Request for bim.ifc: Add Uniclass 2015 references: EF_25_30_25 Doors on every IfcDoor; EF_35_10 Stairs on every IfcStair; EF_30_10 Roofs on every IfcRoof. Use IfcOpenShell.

First a look at what the model holds.

```python
import ifcopenshell

model = ifcopenshell.open("bim.ifc")
print(model.schema)
print("classifications:", [c.Name for c in model.by_type("IfcClassification")])
for ifc_class in ("IfcDoor", "IfcRoof", "IfcStair", "IfcWall", "IfcWindow"):
    print(ifc_class, len(model.by_type(ifc_class)))
```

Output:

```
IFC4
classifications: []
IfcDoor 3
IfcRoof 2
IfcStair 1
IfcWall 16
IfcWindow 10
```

```python
import ifcopenshell
import ifcopenshell.api.classification

model = ifcopenshell.open("bim.ifc")

system = ifcopenshell.api.classification.add_classification(model, classification="Uniclass 2015")

codes = {
    "IfcDoor": ("EF_25_30_25", "Doors"),
    "IfcStair": ("EF_35_10", "Stairs"),
    "IfcRoof": ("EF_30_10", "Roofs"),
}
for ifc_class, (code, name) in codes.items():
    products = model.by_type(ifc_class)
    ifcopenshell.api.classification.add_reference(
        model, products=products, classification=system, identification=code, name=name
    )
    print(code, len(products))

model.write("bim_edited.ifc")
```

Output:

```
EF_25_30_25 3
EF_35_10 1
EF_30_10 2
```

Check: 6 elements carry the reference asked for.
